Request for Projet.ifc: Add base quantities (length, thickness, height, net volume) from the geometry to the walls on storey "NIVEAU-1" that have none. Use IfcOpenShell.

First a look at what the model holds.

```python
import ifcopenshell
import ifcopenshell.util.element
import ifcopenshell.util.unit

model = ifcopenshell.open("Projet.ifc")
print(model.schema)
for unit_type in ("LENGTHUNIT", "AREAUNIT", "VOLUMEUNIT"):
    print(unit_type, ifcopenshell.util.unit.calculate_unit_scale(model, unit_type))
storey = next(s for s in model.by_type("IfcBuildingStorey") if s.Name == "NIVEAU-1")
walls = [e for e in ifcopenshell.util.element.get_decomposition(storey) if e.is_a("IfcWall")]
for e in sorted(walls, key=lambda e: e.id()):
    print(e.id(), e.is_a(), e.Name, list(ifcopenshell.util.element.get_psets(e, qtos_only=True)), sep=" | ")
```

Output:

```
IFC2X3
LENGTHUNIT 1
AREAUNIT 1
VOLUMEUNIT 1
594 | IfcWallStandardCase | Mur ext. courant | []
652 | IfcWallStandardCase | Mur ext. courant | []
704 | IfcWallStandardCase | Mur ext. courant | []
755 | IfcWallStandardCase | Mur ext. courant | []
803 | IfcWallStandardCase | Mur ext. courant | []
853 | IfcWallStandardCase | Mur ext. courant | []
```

```python
import ifcopenshell
import ifcopenshell.api.pset
import ifcopenshell.geom
import ifcopenshell.util.element
import ifcopenshell.util.shape
import ifcopenshell.util.unit

model = ifcopenshell.open("Projet.ifc")
unit_scale = ifcopenshell.util.unit.calculate_unit_scale(model)
volume_scale = ifcopenshell.util.unit.calculate_unit_scale(model, "VOLUMEUNIT")
settings = ifcopenshell.geom.settings()

storey = next(s for s in model.by_type("IfcBuildingStorey") if s.Name == "NIVEAU-1")
walls = [e for e in ifcopenshell.util.element.get_decomposition(storey) if e.is_a("IfcWall")]

for e in sorted(walls, key=lambda e: e.id()):
    if ifcopenshell.util.element.get_psets(e, qtos_only=True, should_inherit=False):
        continue
    # Geometry comes back in metres, in the element's own axes.
    shape = ifcopenshell.geom.create_shape(settings, e)
    values = {
        "Length": ifcopenshell.util.shape.get_x(shape.geometry) / unit_scale,
        "Width": ifcopenshell.util.shape.get_y(shape.geometry) / unit_scale,
        "Height": ifcopenshell.util.shape.get_z(shape.geometry) / unit_scale,
        "NetVolume": ifcopenshell.util.shape.get_volume(shape.geometry) / volume_scale,
    }
    qto = ifcopenshell.api.pset.add_qto(model, product=e, name="BaseQuantities")
    ifcopenshell.api.pset.edit_qto(model, qto=qto, properties=values)
    print(e.id(), {k: round(v, 3) for k, v in values.items()})

model.write("Projet_edited.ifc")
```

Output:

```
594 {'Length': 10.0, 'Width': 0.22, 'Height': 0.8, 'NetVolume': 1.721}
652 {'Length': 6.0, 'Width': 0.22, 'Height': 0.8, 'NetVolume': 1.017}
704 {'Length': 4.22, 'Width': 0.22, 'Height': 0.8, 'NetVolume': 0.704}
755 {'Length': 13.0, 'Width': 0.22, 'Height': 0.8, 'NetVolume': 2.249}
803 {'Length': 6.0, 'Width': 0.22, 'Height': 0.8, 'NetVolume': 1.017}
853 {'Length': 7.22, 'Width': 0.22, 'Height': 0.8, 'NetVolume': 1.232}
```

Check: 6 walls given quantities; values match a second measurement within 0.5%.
